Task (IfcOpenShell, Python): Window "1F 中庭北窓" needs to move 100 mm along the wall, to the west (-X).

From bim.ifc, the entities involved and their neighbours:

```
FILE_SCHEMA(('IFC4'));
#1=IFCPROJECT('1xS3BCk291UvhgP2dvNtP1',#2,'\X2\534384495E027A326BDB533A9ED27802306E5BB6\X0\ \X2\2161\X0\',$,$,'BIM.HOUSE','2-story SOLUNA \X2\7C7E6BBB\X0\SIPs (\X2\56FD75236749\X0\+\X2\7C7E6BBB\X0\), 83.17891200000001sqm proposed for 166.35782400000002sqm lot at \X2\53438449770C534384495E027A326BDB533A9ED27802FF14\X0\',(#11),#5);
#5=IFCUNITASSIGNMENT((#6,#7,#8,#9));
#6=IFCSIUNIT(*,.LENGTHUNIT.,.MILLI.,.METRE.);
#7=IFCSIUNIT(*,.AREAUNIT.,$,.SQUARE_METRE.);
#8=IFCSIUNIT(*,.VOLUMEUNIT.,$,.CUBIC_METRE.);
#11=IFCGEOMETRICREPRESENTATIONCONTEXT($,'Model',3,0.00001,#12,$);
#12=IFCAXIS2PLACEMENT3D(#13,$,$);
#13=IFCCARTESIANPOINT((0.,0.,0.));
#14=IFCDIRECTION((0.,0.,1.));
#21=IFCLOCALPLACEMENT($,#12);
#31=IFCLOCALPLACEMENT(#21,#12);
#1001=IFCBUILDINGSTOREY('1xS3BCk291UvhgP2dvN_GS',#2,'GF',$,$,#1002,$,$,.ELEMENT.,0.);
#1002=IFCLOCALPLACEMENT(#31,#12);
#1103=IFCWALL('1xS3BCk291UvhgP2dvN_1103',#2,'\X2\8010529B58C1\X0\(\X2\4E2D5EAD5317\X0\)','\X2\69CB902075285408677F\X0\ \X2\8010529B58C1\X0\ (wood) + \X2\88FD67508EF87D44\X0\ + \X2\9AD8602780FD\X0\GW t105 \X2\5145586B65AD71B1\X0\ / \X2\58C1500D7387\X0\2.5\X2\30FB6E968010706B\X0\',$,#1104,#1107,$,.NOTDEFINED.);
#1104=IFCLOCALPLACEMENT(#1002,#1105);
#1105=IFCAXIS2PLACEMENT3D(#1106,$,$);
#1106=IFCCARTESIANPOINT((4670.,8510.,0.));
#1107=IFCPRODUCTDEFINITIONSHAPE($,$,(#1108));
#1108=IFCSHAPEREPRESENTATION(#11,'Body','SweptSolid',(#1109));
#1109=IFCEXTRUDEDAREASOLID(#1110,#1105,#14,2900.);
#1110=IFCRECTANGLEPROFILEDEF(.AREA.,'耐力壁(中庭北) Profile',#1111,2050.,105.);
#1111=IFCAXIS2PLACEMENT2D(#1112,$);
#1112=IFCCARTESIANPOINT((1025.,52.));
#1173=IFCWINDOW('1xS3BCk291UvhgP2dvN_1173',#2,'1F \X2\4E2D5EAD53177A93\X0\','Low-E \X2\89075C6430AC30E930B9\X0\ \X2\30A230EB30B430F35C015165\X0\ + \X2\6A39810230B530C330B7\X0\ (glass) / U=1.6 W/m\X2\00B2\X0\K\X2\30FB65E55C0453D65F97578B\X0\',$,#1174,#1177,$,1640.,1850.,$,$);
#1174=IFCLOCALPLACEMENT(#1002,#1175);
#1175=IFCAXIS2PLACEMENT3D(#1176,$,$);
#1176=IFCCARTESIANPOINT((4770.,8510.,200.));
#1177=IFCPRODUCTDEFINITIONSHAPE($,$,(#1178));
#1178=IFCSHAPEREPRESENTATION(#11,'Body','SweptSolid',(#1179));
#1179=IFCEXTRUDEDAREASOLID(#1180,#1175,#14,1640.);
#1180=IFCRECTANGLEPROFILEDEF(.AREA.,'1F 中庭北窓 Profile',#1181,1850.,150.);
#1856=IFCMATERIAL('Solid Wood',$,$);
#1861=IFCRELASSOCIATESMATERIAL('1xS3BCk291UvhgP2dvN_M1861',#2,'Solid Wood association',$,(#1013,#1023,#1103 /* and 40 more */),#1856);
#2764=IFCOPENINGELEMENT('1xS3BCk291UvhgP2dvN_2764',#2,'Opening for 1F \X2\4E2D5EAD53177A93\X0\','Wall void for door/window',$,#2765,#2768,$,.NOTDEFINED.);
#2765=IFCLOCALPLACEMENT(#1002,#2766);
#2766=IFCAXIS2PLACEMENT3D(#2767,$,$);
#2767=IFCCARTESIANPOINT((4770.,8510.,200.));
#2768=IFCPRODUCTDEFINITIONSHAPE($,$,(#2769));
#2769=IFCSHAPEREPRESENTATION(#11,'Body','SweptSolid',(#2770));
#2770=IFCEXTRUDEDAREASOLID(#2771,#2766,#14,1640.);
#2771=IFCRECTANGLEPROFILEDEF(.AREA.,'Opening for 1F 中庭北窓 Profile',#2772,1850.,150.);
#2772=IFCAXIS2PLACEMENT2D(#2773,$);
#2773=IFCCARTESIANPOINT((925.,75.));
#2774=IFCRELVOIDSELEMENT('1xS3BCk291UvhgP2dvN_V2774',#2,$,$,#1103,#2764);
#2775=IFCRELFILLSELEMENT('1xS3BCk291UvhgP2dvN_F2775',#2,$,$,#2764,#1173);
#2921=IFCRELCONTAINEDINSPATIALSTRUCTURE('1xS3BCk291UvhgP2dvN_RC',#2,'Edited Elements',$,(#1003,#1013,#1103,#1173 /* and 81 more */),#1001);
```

```python
import ifcopenshell
import ifcopenshell.api.geometry
import ifcopenshell.util.placement
import ifcopenshell.util.unit

model = ifcopenshell.open("bim.ifc")
unit_scale = ifcopenshell.util.unit.calculate_unit_scale(model)

window = model.by_id(1173)
opening = window.FillsVoids[0].RelatingOpeningElement
wall = opening.VoidsElements[0].RelatingBuildingElement

wall_matrix = ifcopenshell.util.placement.get_local_placement(wall.ObjectPlacement)
shift = wall_matrix[:3, 0] * -0.1 / unit_scale
before = ifcopenshell.util.placement.get_local_placement(window.ObjectPlacement)[:3, 3].copy()

# The window is not placed relative to its opening, so move both.
for product in (opening, window):
    matrix = ifcopenshell.util.placement.get_local_placement(product.ObjectPlacement)
    matrix[:3, 3] += shift
    ifcopenshell.api.geometry.edit_object_placement(model, product=product, matrix=matrix, is_si=False)

after = ifcopenshell.util.placement.get_local_placement(window.ObjectPlacement)[:3, 3]
print("window moved by", (after - before).round(3) + 0.0)

model.write("bim_edited.ifc")
```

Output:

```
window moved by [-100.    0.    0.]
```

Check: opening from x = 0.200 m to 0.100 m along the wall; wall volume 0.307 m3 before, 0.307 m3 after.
